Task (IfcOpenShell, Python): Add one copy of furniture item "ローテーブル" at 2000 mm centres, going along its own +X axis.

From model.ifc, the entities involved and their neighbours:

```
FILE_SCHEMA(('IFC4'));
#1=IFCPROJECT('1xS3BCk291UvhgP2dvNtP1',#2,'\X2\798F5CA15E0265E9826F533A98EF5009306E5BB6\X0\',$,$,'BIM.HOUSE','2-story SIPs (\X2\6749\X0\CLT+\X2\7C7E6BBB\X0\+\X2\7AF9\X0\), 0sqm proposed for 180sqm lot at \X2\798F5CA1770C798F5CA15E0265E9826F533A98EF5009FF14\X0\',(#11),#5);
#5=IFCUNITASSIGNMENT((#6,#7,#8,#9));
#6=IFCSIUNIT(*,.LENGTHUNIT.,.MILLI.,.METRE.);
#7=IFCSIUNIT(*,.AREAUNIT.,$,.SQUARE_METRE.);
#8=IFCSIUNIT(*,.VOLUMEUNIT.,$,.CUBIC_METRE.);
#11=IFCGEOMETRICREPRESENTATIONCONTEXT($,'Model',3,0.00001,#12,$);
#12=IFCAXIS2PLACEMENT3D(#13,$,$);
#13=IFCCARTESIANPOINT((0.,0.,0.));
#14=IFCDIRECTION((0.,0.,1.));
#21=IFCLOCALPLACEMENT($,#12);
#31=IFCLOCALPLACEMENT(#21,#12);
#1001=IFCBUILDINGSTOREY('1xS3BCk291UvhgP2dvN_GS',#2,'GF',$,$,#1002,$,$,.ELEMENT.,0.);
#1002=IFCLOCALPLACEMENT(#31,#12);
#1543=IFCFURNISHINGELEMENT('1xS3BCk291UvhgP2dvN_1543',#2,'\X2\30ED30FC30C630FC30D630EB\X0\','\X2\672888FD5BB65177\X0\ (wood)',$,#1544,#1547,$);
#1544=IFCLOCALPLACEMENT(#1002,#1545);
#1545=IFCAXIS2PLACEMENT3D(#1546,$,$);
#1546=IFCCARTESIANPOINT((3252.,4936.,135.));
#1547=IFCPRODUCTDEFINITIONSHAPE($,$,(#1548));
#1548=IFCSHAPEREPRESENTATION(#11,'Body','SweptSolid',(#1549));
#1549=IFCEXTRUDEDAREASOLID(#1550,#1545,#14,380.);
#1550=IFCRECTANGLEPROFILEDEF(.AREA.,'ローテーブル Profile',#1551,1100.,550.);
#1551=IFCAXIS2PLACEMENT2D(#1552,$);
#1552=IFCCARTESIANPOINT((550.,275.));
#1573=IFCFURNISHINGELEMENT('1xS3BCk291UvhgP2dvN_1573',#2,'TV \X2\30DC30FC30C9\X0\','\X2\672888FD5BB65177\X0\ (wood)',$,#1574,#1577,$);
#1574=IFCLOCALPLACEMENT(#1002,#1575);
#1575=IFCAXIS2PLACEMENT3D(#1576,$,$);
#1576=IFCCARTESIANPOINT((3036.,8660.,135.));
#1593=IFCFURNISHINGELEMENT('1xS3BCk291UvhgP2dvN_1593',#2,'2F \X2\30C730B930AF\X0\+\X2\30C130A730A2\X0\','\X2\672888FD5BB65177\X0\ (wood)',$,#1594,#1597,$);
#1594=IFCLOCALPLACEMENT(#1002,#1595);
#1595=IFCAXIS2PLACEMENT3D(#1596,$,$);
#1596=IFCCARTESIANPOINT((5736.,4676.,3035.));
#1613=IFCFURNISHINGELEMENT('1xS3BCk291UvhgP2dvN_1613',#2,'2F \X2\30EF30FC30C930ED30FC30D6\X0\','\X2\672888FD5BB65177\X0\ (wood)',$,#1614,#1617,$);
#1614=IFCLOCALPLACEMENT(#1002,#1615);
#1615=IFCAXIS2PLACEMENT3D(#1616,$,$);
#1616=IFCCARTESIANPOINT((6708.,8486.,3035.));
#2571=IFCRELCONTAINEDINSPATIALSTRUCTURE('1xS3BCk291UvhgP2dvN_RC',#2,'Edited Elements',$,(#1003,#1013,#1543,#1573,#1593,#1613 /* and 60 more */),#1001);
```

```python
import ifcopenshell
import ifcopenshell.api.geometry
import ifcopenshell.api.root
import ifcopenshell.util.element
import ifcopenshell.util.placement
import ifcopenshell.util.unit

model = ifcopenshell.open("model.ifc")
unit_scale = ifcopenshell.util.unit.calculate_unit_scale(model)


def reuse_history(source, copy):
    """copy_class also copies each property set's owner history, people and application; keep the originals."""
    for rel in copy.IsDefinedBy:
        if rel.is_a("IfcRelDefinesByProperties") and (history := rel.RelatingPropertyDefinition.OwnerHistory):
            rel.RelatingPropertyDefinition.OwnerHistory = source.OwnerHistory
            ifcopenshell.util.element.remove_deep2(model, history)


source = model.by_guid("1xS3BCk291UvhgP2dvN_1543")
base = ifcopenshell.util.placement.get_local_placement(source.ObjectPlacement)
step = base[:3, 0] * 2 / unit_scale

for i in range(1, 2):
    copy = ifcopenshell.api.root.copy_class(model, product=source)
    copy.Representation = ifcopenshell.util.element.copy_deep(
        model, source.Representation, exclude=["IfcGeometricRepresentationContext", "IfcRepresentationMap"]
    )
    reuse_history(source, copy)
    matrix = base.copy()
    matrix[:3, 3] += i * step
    print("added at", matrix[:3, 3].round(3) + 0.0)
    ifcopenshell.api.geometry.edit_object_placement(model, product=copy, matrix=matrix, is_si=False)

model.write("model_updated.ifc")
```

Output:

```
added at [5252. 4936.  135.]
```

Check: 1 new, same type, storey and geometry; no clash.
